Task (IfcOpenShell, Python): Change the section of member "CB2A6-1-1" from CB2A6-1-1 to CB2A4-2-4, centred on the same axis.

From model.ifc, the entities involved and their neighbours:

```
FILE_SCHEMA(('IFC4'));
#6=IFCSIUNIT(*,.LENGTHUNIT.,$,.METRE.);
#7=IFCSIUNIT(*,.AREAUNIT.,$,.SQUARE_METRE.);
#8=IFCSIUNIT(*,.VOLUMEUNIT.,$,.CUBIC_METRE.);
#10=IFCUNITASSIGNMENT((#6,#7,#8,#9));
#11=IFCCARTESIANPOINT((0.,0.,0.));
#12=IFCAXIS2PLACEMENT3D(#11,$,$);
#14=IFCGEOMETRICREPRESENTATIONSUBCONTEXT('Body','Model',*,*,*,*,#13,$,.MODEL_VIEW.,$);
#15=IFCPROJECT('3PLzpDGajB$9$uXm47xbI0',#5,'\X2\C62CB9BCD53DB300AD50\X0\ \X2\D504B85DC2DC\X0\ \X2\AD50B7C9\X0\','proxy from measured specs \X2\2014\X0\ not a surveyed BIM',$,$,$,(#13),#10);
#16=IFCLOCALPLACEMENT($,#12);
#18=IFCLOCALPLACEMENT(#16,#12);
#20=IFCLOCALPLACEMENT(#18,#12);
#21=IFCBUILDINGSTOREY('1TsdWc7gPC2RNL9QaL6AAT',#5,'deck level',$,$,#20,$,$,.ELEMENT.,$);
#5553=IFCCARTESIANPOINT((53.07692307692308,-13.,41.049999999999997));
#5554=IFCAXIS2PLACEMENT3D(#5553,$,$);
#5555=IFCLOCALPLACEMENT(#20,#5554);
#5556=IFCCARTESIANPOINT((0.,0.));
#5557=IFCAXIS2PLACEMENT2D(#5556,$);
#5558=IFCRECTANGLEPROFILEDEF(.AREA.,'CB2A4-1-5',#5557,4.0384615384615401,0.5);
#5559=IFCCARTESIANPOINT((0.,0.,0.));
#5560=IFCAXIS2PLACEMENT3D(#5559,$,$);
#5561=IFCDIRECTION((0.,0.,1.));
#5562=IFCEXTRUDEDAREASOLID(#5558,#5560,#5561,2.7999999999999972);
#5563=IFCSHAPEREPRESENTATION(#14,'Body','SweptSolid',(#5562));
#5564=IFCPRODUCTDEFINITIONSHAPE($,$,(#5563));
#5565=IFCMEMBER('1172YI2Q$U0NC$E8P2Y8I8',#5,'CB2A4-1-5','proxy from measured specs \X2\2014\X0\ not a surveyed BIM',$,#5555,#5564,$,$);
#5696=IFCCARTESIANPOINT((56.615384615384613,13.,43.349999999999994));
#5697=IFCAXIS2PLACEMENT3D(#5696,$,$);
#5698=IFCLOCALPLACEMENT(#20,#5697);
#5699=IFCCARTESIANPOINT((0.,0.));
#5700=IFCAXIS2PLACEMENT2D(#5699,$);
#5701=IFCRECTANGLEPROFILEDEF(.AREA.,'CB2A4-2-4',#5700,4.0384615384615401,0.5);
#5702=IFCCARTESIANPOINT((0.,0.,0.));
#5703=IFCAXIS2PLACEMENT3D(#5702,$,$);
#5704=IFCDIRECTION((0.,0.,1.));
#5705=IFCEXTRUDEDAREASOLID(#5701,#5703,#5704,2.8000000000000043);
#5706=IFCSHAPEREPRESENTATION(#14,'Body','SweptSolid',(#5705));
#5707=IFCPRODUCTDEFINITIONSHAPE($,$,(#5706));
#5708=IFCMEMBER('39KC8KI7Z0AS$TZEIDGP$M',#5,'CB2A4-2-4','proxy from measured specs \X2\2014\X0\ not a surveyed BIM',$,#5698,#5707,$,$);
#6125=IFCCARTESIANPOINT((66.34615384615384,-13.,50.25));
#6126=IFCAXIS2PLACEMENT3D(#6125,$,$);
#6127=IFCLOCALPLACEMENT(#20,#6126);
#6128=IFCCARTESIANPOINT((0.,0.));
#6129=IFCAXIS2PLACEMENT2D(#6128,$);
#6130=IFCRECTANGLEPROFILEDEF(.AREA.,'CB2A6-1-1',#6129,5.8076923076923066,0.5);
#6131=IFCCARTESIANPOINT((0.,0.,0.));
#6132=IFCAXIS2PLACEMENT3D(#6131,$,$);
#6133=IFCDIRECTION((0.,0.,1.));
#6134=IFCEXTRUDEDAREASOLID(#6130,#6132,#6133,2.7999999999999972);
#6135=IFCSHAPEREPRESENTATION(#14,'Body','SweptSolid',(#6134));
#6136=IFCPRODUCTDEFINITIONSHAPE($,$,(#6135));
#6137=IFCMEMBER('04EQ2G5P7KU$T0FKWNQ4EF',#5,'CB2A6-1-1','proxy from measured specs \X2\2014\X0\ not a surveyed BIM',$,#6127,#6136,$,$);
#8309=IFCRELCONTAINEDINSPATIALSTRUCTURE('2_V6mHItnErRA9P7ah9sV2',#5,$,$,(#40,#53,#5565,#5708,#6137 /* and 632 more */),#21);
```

```python
import ifcopenshell
import ifcopenshell.util.element
import ifcopenshell.util.representation

model = ifcopenshell.open("model.ifc")

member = model.by_id(6137)
source = next(p for p in model.by_type("IfcRectangleProfileDef") if p.ProfileName == "CB2A4-2-4")

body = ifcopenshell.util.representation.get_representation(member, "Model", "Body")
solid = body.Items[0]
old_profile = solid.SweptArea

# Copy the section's sizes but keep this member's own profile position.
profile = ifcopenshell.util.element.copy(model, source)
profile.Position = old_profile.Position
solid.SweptArea = profile
if not model.get_total_inverses(old_profile):
    ifcopenshell.util.element.remove_deep2(model, old_profile)
member.Name = member.Name.replace("CB2A6-1-1", "CB2A4-2-4")

print(solid.SweptArea)

model.write("model-out.ifc")
```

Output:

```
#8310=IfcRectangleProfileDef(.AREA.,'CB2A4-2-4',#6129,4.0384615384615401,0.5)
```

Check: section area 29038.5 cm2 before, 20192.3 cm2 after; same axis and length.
